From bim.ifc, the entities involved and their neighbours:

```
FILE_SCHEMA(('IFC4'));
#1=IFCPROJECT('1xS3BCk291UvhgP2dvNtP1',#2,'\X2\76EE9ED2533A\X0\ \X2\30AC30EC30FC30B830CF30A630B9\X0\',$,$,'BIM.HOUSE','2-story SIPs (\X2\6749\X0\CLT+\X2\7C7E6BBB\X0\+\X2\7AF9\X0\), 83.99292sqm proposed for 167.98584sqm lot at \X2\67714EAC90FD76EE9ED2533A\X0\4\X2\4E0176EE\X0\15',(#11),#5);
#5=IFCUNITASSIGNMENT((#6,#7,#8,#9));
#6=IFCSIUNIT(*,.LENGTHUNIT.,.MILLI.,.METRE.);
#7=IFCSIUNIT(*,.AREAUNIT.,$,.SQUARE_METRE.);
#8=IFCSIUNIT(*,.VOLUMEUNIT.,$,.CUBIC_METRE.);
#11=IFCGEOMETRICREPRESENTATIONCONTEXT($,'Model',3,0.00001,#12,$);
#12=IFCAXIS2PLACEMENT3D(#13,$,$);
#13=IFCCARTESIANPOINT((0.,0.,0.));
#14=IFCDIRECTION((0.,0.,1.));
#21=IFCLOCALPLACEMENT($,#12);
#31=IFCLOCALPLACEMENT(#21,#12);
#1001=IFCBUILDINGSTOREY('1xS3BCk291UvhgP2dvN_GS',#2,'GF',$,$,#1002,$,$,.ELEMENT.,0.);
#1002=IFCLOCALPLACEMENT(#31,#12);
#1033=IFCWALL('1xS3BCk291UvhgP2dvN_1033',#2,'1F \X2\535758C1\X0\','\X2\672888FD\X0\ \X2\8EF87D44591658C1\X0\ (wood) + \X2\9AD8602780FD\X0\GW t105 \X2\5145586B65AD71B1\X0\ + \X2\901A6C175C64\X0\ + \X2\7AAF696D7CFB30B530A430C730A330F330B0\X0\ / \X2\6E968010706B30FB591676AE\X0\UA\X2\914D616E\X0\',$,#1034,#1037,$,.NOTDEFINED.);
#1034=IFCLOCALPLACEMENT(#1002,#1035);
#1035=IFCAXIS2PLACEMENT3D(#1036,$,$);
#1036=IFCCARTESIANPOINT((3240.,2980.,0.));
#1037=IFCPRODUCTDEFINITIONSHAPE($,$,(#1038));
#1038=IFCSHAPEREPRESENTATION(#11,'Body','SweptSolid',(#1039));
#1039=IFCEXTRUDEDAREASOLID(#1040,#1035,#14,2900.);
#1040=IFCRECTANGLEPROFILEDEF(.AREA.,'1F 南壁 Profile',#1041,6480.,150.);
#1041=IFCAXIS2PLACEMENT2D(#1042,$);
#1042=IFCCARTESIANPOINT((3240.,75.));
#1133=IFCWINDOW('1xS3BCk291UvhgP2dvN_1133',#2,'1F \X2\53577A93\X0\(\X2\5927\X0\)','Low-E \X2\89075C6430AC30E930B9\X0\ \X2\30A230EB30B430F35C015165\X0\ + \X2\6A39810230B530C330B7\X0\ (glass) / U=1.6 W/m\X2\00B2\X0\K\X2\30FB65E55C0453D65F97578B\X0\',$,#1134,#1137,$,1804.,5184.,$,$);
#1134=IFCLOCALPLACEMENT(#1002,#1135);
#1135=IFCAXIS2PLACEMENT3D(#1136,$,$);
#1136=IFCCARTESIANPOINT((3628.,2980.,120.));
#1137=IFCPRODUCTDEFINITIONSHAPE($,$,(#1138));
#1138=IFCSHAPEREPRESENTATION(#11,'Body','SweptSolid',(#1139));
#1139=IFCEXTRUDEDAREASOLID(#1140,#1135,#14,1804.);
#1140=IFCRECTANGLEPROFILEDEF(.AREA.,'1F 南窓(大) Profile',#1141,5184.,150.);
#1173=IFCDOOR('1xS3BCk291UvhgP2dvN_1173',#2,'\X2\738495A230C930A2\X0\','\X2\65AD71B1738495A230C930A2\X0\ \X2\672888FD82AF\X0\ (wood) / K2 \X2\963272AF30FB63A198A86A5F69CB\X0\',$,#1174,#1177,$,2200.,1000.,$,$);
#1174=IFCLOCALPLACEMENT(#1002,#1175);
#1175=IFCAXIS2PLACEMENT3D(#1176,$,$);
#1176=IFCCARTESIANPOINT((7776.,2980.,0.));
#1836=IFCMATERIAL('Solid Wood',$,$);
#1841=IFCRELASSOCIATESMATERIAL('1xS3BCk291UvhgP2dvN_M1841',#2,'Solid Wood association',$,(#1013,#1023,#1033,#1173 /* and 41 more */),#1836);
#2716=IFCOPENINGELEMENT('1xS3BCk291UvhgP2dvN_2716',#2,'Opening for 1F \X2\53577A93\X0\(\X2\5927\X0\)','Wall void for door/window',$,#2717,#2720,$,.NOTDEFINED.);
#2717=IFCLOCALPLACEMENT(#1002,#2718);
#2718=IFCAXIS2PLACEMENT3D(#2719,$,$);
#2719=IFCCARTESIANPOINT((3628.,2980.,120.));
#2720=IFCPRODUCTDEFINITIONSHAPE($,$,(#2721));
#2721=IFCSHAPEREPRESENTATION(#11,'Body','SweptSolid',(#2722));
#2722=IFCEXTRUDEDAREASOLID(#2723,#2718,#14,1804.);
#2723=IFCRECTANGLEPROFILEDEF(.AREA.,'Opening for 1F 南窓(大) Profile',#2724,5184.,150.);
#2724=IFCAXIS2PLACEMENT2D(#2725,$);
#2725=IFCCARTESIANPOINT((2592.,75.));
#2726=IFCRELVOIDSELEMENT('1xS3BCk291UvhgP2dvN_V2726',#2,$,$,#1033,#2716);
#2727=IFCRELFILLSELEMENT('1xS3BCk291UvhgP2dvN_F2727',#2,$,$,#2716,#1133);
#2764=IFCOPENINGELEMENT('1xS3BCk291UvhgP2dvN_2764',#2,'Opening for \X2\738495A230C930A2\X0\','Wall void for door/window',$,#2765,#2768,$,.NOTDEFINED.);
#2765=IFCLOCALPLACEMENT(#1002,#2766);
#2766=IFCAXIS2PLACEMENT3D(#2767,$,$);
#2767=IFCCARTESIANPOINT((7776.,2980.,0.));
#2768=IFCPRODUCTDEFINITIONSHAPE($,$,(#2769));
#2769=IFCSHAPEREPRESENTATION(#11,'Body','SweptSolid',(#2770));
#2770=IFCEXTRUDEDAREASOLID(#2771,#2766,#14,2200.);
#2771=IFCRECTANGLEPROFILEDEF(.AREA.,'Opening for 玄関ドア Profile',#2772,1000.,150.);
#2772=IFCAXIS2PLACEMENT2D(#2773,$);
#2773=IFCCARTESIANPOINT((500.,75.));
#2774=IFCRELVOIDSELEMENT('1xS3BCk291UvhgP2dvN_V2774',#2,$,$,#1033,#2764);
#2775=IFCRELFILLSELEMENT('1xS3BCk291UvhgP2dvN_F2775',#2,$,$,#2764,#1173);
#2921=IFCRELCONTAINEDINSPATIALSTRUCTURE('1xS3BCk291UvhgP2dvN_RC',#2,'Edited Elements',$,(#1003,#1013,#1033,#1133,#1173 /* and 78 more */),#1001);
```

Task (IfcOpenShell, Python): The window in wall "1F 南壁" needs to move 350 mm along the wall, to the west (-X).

```python
import ifcopenshell
import ifcopenshell.api.geometry
import ifcopenshell.util.placement
import ifcopenshell.util.unit

model = ifcopenshell.open("bim.ifc")
unit_scale = ifcopenshell.util.unit.calculate_unit_scale(model)

window = model.by_id(1133)
opening = window.FillsVoids[0].RelatingOpeningElement
wall = opening.VoidsElements[0].RelatingBuildingElement

wall_matrix = ifcopenshell.util.placement.get_local_placement(wall.ObjectPlacement)
shift = wall_matrix[:3, 0] * -0.35 / unit_scale
before = ifcopenshell.util.placement.get_local_placement(window.ObjectPlacement)[:3, 3].copy()

# The window is not placed relative to its opening, so move both.
for product in (opening, window):
    matrix = ifcopenshell.util.placement.get_local_placement(product.ObjectPlacement)
    matrix[:3, 3] += shift
    ifcopenshell.api.geometry.edit_object_placement(model, product=product, matrix=matrix, is_si=False)

after = ifcopenshell.util.placement.get_local_placement(window.ObjectPlacement)[:3, 3]
print("window moved by", (after - before).round(3) + 0.0)

model.write("bim_v2.ifc")
```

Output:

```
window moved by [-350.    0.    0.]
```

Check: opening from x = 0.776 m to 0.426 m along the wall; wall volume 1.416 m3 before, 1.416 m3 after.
